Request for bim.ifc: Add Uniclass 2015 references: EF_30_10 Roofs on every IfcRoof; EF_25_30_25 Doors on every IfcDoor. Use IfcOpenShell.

First a look at what the model holds.

```python
import ifcopenshell

model = ifcopenshell.open("bim.ifc")
print(model.schema)
print("classifications:", [c.Name for c in model.by_type("IfcClassification")])
for ifc_class in ("IfcDoor", "IfcRoof", "IfcStair", "IfcWall", "IfcWindow"):
    print(ifc_class, len(model.by_type(ifc_class)))
```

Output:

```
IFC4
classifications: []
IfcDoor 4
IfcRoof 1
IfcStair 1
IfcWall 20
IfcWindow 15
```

```python
import ifcopenshell
import ifcopenshell.api.classification

model = ifcopenshell.open("bim.ifc")

system = ifcopenshell.api.classification.add_classification(model, classification="Uniclass 2015")

codes = {
    "IfcRoof": ("EF_30_10", "Roofs"),
    "IfcDoor": ("EF_25_30_25", "Doors"),
}
for ifc_class, (code, name) in codes.items():
    products = model.by_type(ifc_class)
    ifcopenshell.api.classification.add_reference(
        model, products=products, classification=system, identification=code, name=name
    )
    print(code, len(products))

model.write("bim_updated.ifc")
```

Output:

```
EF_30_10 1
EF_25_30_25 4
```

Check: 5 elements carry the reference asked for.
